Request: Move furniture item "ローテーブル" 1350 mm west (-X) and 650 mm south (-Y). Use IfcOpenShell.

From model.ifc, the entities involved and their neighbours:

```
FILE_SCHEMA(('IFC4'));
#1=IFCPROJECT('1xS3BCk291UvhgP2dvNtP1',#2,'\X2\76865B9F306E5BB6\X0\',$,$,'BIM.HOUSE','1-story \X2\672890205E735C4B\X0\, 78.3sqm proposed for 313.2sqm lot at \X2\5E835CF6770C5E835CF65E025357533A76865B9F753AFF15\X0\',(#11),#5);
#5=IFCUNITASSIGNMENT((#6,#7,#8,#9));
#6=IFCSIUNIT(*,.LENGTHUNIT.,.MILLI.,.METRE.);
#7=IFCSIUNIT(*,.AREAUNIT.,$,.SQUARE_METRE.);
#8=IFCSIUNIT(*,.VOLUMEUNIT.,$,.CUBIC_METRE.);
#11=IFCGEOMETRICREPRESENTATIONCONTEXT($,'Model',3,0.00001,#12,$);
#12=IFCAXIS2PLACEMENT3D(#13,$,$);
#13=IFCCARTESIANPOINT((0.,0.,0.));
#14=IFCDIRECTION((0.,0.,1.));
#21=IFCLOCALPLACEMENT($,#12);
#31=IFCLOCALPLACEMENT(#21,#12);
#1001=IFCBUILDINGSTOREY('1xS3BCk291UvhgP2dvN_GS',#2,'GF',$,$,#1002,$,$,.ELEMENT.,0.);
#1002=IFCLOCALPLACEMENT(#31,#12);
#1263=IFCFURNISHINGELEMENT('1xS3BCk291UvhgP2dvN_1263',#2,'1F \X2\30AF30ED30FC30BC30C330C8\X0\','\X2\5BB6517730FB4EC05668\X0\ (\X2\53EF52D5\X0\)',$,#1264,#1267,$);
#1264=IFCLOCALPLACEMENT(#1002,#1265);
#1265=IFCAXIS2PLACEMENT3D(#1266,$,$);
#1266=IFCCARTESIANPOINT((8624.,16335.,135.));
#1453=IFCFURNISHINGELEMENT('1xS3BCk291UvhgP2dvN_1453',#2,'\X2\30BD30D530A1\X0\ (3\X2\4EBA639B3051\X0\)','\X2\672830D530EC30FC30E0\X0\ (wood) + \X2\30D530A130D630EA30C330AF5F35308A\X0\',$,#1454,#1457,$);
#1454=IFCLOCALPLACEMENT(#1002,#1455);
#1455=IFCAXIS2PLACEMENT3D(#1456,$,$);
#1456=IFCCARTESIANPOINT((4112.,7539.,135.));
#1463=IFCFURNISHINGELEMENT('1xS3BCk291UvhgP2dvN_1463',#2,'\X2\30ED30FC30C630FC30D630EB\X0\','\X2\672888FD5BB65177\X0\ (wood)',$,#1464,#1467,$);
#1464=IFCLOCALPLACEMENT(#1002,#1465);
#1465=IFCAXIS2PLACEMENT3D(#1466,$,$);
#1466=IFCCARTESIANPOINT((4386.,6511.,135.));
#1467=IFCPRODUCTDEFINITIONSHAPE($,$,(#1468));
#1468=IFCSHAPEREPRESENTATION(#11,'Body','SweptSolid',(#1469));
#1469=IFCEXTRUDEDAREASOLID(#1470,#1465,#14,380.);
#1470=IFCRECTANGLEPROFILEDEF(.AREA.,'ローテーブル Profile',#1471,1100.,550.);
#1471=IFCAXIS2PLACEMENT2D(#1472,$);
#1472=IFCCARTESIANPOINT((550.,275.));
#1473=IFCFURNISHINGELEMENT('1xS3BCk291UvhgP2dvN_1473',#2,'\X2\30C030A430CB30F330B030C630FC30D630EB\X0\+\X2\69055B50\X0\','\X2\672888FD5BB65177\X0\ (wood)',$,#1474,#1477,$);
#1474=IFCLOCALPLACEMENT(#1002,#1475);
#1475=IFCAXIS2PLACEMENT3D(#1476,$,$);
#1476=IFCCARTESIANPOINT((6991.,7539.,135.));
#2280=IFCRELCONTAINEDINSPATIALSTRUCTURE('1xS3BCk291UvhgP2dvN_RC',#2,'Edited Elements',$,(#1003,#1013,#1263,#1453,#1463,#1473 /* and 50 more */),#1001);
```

```python
import ifcopenshell
import ifcopenshell.api.geometry
import ifcopenshell.util.placement
import ifcopenshell.util.unit

model = ifcopenshell.open("model.ifc")
unit_scale = ifcopenshell.util.unit.calculate_unit_scale(model)

item = model.by_id(1463)
matrix = ifcopenshell.util.placement.get_local_placement(item.ObjectPlacement)
matrix[0, 3] -= 1.35 / unit_scale
matrix[1, 3] -= 0.65 / unit_scale
ifcopenshell.api.geometry.edit_object_placement(model, product=item, matrix=matrix, is_si=False)

print(ifcopenshell.util.placement.get_local_placement(item.ObjectPlacement).round(3) + 0.0)

model.write("model_edited.ifc")
```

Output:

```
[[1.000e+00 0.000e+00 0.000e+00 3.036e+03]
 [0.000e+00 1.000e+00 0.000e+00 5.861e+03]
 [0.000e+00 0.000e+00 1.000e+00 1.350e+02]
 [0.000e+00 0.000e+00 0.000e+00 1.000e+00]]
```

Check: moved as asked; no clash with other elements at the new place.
